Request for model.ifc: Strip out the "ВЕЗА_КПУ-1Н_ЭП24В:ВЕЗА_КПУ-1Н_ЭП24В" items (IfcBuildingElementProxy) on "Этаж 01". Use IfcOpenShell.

First a look at what the model holds.

```python
import ifcopenshell
import ifcopenshell.util.element

model = ifcopenshell.open("model.ifc")
print(model.schema)
storey = next(s for s in model.by_type("IfcBuildingStorey") if s.Name == "Этаж 01")
proxies = [e for e in ifcopenshell.util.element.get_decomposition(storey) if e.is_a("IfcBuildingElementProxy")]
seen = {}
for e in proxies:
    element_type = ifcopenshell.util.element.get_type(e)
    name = element_type.Name if element_type not in (None, e) else None
    seen[name] = seen.get(name, 0) + 1
for name, count in sorted(seen.items(), key=str):
    print(count, "x", name)
```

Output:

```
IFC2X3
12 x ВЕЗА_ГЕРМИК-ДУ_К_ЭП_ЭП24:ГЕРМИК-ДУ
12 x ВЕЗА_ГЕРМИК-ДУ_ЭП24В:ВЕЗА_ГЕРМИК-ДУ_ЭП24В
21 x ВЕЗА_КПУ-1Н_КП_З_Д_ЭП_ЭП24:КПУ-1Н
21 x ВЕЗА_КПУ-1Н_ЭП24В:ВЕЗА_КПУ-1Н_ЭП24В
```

```python
import ifcopenshell
import ifcopenshell.api.root
import ifcopenshell.util.element

model = ifcopenshell.open("model.ifc")

storey = next(s for s in model.by_type("IfcBuildingStorey") if s.Name == "Этаж 01")
proxies = [e for e in ifcopenshell.util.element.get_decomposition(storey) if e.is_a("IfcBuildingElementProxy")]
targets = [e for e in proxies if (t := ifcopenshell.util.element.get_type(e)) not in (None, e) and t.Name == "ВЕЗА_КПУ-1Н_ЭП24В:ВЕЗА_КПУ-1Н_ЭП24В"]

for e in targets:
    ifcopenshell.api.root.remove_product(model, product=e)
print(len(targets), "removed")

model.write("model-out.ifc")
```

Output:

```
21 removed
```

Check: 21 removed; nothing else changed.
